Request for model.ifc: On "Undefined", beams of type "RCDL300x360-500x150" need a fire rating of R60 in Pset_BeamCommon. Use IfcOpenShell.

First a look at what the model holds.

```python
import ifcopenshell
import ifcopenshell.util.element

model = ifcopenshell.open("model.ifc")
print(model.schema)
storey = next(s for s in model.by_type("IfcBuildingStorey") if s.Name == "Undefined")
beams = [e for e in ifcopenshell.util.element.get_decomposition(storey) if e.is_a("IfcBeam")]
seen = {}
for e in beams:
    element_type = ifcopenshell.util.element.get_type(e)
    key = (element_type.Name if element_type != e and element_type else None, ifcopenshell.util.element.get_pset(e, "Pset_BeamCommon", "FireRating"))
    seen[key] = seen.get(key, 0) + 1
for (name, value), count in sorted(seen.items(), key=str):
    print(count, "x", name, "|", value)
```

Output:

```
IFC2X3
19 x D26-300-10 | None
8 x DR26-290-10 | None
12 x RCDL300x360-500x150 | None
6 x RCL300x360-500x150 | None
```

```python
import ifcopenshell
import ifcopenshell.api.pset
import ifcopenshell.util.element

model = ifcopenshell.open("model.ifc")

storey = next(s for s in model.by_type("IfcBuildingStorey") if s.Name == "Undefined")
beams = [e for e in ifcopenshell.util.element.get_decomposition(storey) if e.is_a("IfcBeam")]

count = 0
for e in beams:
    element_type = ifcopenshell.util.element.get_type(e)
    if element_type in (None, e) or element_type.Name != "RCDL300x360-500x150":
        continue
    found = ifcopenshell.util.element.get_pset(e, "Pset_BeamCommon", should_inherit=False)
    if found:
        pset = model.by_id(found["id"])
        if len(ifcopenshell.util.element.get_elements_by_pset(pset)) > 1:
            pset = ifcopenshell.api.pset.unshare_pset(model, products=[e], pset=pset)[0]
    else:
        pset = ifcopenshell.api.pset.add_pset(model, product=e, name="Pset_BeamCommon")
    ifcopenshell.api.pset.edit_pset(model, pset=pset, properties={"FireRating": "R60"})
    count += 1

print(count, "beams updated")

model.write("model-out.ifc")
```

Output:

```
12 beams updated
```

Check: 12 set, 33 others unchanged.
